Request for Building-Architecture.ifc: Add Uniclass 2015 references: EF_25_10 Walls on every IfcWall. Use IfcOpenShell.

First a look at what the model holds.

```python
import ifcopenshell

model = ifcopenshell.open("Building-Architecture.ifc")
print(model.schema)
print("classifications:", [c.Name for c in model.by_type("IfcClassification")])
for ifc_class in ("IfcDoor", "IfcRoof", "IfcStair", "IfcWall", "IfcWindow"):
    print(ifc_class, len(model.by_type(ifc_class)))
```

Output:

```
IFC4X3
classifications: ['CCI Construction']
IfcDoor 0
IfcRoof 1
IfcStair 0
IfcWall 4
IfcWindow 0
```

```python
import ifcopenshell
import ifcopenshell.api.classification

model = ifcopenshell.open("Building-Architecture.ifc")

system = ifcopenshell.api.classification.add_classification(model, classification="Uniclass 2015")

codes = {
    "IfcWall": ("EF_25_10", "Walls"),
}
for ifc_class, (code, name) in codes.items():
    products = model.by_type(ifc_class)
    ifcopenshell.api.classification.add_reference(
        model, products=products, classification=system, identification=code, name=name
    )
    print(code, len(products))

model.write("Building-Architecture_updated.ifc")
```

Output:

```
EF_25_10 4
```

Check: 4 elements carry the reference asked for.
